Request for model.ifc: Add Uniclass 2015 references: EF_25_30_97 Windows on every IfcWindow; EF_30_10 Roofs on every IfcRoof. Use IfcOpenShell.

First a look at what the model holds.

```python
import ifcopenshell

model = ifcopenshell.open("model.ifc")
print(model.schema)
print("classifications:", [c.Name for c in model.by_type("IfcClassification")])
for ifc_class in ("IfcDoor", "IfcRoof", "IfcStair", "IfcWall", "IfcWindow"):
    print(ifc_class, len(model.by_type(ifc_class)))
```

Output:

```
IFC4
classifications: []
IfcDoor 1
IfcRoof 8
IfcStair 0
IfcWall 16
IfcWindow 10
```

```python
import ifcopenshell
import ifcopenshell.api.classification

model = ifcopenshell.open("model.ifc")

system = ifcopenshell.api.classification.add_classification(model, classification="Uniclass 2015")

codes = {
    "IfcWindow": ("EF_25_30_97", "Windows"),
    "IfcRoof": ("EF_30_10", "Roofs"),
}
for ifc_class, (code, name) in codes.items():
    products = model.by_type(ifc_class)
    ifcopenshell.api.classification.add_reference(
        model, products=products, classification=system, identification=code, name=name
    )
    print(code, len(products))

model.write("model_updated.ifc")
```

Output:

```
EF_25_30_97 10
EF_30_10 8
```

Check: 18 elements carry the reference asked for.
